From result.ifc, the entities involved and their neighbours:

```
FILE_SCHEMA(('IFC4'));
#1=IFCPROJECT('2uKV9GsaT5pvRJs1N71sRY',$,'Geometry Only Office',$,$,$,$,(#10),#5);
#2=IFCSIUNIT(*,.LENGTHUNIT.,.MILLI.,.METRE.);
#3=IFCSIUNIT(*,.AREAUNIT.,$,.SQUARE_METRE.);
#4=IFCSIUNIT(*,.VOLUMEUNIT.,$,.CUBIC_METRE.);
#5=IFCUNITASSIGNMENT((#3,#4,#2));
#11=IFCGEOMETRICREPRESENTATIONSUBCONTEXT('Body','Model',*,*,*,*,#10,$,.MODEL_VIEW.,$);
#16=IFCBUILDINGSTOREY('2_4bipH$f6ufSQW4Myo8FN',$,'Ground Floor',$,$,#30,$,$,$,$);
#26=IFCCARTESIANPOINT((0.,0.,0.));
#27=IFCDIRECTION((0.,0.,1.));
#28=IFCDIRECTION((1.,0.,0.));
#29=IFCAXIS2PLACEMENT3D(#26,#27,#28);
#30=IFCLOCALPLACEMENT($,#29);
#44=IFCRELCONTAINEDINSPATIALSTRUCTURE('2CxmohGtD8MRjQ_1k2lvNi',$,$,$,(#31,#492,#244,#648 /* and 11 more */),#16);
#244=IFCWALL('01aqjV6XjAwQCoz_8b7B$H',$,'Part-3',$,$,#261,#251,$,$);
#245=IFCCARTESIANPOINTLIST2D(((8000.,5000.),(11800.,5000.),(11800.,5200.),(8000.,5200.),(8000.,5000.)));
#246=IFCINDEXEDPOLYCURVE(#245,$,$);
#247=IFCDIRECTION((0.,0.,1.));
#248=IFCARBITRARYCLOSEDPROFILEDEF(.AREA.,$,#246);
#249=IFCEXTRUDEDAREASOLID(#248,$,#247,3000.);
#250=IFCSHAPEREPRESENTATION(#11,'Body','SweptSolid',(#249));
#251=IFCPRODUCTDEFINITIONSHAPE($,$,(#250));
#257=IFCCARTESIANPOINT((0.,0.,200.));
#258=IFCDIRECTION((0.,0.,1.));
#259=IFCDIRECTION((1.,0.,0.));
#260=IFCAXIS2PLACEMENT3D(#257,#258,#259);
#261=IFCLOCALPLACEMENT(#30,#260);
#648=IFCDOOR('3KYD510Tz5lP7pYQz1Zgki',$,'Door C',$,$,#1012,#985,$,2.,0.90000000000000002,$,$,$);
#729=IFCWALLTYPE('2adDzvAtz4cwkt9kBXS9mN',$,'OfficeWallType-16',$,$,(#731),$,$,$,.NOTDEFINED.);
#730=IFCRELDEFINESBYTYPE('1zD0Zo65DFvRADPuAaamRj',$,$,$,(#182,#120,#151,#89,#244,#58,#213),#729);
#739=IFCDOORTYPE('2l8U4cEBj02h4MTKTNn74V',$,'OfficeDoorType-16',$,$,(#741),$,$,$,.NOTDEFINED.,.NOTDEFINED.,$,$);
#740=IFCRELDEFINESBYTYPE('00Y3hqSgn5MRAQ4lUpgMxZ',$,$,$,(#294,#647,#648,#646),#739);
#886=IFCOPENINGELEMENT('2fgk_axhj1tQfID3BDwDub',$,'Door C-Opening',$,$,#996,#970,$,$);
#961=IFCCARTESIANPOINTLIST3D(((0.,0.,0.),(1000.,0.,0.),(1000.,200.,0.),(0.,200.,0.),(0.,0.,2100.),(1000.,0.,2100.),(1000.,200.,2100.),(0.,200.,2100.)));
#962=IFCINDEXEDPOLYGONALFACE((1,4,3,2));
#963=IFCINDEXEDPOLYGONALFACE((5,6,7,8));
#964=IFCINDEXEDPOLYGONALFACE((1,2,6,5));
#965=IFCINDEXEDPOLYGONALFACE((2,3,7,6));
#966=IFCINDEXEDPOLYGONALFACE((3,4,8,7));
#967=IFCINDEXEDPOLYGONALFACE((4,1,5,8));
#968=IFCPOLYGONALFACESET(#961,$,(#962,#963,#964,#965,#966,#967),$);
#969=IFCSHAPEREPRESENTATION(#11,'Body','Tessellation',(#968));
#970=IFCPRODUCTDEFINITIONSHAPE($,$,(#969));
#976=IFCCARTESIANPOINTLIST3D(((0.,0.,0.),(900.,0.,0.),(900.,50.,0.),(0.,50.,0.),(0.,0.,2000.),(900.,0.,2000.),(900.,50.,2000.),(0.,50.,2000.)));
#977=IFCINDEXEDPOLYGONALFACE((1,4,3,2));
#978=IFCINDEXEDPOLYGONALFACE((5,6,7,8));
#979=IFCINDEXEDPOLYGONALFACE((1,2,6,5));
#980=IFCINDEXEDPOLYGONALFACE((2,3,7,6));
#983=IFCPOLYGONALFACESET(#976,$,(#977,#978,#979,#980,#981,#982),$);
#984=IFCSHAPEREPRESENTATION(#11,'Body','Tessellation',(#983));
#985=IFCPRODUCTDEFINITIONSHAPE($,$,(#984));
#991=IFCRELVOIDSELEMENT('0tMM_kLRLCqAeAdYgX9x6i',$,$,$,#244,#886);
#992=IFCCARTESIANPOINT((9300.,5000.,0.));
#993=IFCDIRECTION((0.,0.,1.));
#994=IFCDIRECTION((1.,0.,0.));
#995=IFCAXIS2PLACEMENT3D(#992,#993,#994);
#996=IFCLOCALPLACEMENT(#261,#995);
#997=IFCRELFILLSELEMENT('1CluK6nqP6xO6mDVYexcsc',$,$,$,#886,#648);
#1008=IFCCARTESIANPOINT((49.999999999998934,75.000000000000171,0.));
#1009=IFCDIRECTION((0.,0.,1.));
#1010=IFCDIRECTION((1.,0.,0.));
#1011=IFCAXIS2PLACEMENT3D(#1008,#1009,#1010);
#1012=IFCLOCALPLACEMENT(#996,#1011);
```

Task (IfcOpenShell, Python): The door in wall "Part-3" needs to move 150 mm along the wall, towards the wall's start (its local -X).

```python
import ifcopenshell
import ifcopenshell.api.geometry
import ifcopenshell.util.placement
import ifcopenshell.util.unit

model = ifcopenshell.open("result.ifc")
unit_scale = ifcopenshell.util.unit.calculate_unit_scale(model)

door = model.by_guid("3KYD510Tz5lP7pYQz1Zgki")
opening = door.FillsVoids[0].RelatingOpeningElement
wall = opening.VoidsElements[0].RelatingBuildingElement

wall_matrix = ifcopenshell.util.placement.get_local_placement(wall.ObjectPlacement)
shift = wall_matrix[:3, 0] * -0.15 / unit_scale
before = ifcopenshell.util.placement.get_local_placement(door.ObjectPlacement)[:3, 3].copy()

# The door is placed relative to its opening, so it follows when the opening moves.
matrix = ifcopenshell.util.placement.get_local_placement(opening.ObjectPlacement)
matrix[:3, 3] += shift
ifcopenshell.api.geometry.edit_object_placement(
    model, product=opening, matrix=matrix, is_si=False, should_transform_children=True
)

after = ifcopenshell.util.placement.get_local_placement(door.ObjectPlacement)[:3, 3]
print("door moved by", (after - before).round(3) + 0.0)

model.write("result-out.ifc")
```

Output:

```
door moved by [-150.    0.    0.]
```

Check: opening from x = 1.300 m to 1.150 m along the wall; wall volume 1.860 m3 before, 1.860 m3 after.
